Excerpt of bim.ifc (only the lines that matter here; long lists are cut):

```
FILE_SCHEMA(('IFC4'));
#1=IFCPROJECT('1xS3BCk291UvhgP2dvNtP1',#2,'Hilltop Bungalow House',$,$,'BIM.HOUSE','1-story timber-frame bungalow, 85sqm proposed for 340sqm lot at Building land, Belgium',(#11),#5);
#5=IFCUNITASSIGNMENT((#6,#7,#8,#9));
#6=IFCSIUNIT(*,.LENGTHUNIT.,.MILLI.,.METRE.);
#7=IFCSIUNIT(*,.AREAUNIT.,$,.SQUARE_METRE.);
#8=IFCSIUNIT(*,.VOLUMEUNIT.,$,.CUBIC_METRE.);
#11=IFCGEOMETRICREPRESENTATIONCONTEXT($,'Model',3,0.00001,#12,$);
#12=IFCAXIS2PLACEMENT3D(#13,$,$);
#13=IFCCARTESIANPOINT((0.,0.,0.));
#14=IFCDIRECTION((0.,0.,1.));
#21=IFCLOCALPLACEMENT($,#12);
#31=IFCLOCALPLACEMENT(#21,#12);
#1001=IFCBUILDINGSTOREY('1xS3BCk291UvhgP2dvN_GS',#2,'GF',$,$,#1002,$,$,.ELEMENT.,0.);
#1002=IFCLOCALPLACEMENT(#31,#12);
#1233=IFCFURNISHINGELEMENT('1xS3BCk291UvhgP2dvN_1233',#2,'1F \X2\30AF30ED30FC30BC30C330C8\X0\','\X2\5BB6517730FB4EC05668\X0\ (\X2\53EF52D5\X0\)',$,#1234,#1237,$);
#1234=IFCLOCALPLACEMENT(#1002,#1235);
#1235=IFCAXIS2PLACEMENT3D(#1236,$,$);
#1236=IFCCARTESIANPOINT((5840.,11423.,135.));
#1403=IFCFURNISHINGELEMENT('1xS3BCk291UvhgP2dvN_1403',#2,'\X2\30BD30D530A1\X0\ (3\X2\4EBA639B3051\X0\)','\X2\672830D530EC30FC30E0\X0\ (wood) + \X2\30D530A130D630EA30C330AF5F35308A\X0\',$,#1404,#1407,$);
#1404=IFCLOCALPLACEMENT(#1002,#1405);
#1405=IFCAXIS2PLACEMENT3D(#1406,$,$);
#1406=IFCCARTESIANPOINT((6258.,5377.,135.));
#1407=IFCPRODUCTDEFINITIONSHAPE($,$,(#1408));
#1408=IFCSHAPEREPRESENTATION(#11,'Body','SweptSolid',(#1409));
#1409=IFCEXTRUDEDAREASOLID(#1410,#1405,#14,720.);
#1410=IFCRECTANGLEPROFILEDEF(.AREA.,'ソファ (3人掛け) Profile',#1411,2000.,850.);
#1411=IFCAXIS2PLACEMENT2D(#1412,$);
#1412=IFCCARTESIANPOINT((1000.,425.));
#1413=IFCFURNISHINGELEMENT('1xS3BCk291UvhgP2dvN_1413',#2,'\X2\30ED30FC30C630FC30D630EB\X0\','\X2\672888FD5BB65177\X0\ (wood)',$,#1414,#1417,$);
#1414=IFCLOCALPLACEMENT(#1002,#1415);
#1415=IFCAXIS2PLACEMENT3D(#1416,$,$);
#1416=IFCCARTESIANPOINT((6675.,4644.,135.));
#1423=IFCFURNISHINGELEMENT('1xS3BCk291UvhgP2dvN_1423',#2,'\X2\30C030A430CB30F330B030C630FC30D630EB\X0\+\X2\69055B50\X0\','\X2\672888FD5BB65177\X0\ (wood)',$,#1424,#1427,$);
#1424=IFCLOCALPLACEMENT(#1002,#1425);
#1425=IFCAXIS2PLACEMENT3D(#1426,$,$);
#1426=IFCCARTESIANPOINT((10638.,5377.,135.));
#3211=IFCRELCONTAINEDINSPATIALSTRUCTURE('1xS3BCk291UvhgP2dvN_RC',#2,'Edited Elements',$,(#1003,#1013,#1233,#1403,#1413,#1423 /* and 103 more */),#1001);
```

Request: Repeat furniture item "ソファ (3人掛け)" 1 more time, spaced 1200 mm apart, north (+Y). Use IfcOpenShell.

```python
import numpy as np
import ifcopenshell
import ifcopenshell.api.geometry
import ifcopenshell.api.root
import ifcopenshell.util.element
import ifcopenshell.util.placement
import ifcopenshell.util.unit

model = ifcopenshell.open("bim.ifc")
unit_scale = ifcopenshell.util.unit.calculate_unit_scale(model)


def reuse_history(source, copy):
    """copy_class also copies each property set's owner history, people and application; keep the originals."""
    for rel in copy.IsDefinedBy:
        if rel.is_a("IfcRelDefinesByProperties") and (history := rel.RelatingPropertyDefinition.OwnerHistory):
            rel.RelatingPropertyDefinition.OwnerHistory = source.OwnerHistory
            ifcopenshell.util.element.remove_deep2(model, history)


source = model.by_guid("1xS3BCk291UvhgP2dvN_1403")
base = ifcopenshell.util.placement.get_local_placement(source.ObjectPlacement)
step = np.array([0.0, 1.0, 0.0]) * 1.2 / unit_scale

for i in range(1, 2):
    copy = ifcopenshell.api.root.copy_class(model, product=source)
    copy.Representation = ifcopenshell.util.element.copy_deep(
        model, source.Representation, exclude=["IfcGeometricRepresentationContext", "IfcRepresentationMap"]
    )
    reuse_history(source, copy)
    matrix = base.copy()
    matrix[:3, 3] += i * step
    print("added at", matrix[:3, 3].round(3) + 0.0)
    ifcopenshell.api.geometry.edit_object_placement(model, product=copy, matrix=matrix, is_si=False)

model.write("bim_edited.ifc")
```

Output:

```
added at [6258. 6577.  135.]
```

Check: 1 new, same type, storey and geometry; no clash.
